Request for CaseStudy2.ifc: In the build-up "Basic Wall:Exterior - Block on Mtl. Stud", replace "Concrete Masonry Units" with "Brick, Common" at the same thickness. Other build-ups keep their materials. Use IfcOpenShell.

First a look at what the model holds.

```python
import ifcopenshell
import ifcopenshell.util.element

model = ifcopenshell.open("CaseStudy2.ifc")
print(model.schema)
for layer_set in model.by_type("IfcMaterialLayerSet"):
    if layer_set.LayerSetName == "Basic Wall:Exterior - Block on Mtl. Stud":
        for layer in layer_set.MaterialLayers:
            print(layer.id(), layer.Material and layer.Material.Name, layer.LayerThickness, sep=" | ")
        print(len(ifcopenshell.util.element.get_elements_by_material(model, layer_set)), "elements and types use it")
print(sorted(m.Name for m in model.by_type("IfcMaterial") if m.Name)[:60])
```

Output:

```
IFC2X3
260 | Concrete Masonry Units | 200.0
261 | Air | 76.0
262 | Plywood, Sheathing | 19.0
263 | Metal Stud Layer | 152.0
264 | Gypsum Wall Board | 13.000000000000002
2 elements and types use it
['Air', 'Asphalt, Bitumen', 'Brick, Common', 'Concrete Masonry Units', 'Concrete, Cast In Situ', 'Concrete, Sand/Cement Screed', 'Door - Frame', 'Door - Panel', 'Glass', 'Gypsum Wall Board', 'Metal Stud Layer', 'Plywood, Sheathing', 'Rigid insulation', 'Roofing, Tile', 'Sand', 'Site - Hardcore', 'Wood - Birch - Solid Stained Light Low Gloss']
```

```python
import ifcopenshell
import ifcopenshell.api.material

model = ifcopenshell.open("CaseStudy2.ifc")

layer_set = next(s for s in model.by_type("IfcMaterialLayerSet") if s.LayerSetName == "Basic Wall:Exterior - Block on Mtl. Stud")
layer = next(l for l in layer_set.MaterialLayers if l.Material and l.Material.Name == "Concrete Masonry Units")
material = next(m for m in model.by_type("IfcMaterial") if m.Name == "Brick, Common")

# Point this one layer at the other material; renaming the old one would change it everywhere.
ifcopenshell.api.material.edit_layer(model, layer=layer, attributes={}, material=material)

print([l.Material.Name if l.Material else None for l in layer_set.MaterialLayers])

model.write("CaseStudy2_updated.ifc")
```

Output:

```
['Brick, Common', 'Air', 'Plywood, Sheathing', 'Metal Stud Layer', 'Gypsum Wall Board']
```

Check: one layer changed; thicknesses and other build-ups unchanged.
